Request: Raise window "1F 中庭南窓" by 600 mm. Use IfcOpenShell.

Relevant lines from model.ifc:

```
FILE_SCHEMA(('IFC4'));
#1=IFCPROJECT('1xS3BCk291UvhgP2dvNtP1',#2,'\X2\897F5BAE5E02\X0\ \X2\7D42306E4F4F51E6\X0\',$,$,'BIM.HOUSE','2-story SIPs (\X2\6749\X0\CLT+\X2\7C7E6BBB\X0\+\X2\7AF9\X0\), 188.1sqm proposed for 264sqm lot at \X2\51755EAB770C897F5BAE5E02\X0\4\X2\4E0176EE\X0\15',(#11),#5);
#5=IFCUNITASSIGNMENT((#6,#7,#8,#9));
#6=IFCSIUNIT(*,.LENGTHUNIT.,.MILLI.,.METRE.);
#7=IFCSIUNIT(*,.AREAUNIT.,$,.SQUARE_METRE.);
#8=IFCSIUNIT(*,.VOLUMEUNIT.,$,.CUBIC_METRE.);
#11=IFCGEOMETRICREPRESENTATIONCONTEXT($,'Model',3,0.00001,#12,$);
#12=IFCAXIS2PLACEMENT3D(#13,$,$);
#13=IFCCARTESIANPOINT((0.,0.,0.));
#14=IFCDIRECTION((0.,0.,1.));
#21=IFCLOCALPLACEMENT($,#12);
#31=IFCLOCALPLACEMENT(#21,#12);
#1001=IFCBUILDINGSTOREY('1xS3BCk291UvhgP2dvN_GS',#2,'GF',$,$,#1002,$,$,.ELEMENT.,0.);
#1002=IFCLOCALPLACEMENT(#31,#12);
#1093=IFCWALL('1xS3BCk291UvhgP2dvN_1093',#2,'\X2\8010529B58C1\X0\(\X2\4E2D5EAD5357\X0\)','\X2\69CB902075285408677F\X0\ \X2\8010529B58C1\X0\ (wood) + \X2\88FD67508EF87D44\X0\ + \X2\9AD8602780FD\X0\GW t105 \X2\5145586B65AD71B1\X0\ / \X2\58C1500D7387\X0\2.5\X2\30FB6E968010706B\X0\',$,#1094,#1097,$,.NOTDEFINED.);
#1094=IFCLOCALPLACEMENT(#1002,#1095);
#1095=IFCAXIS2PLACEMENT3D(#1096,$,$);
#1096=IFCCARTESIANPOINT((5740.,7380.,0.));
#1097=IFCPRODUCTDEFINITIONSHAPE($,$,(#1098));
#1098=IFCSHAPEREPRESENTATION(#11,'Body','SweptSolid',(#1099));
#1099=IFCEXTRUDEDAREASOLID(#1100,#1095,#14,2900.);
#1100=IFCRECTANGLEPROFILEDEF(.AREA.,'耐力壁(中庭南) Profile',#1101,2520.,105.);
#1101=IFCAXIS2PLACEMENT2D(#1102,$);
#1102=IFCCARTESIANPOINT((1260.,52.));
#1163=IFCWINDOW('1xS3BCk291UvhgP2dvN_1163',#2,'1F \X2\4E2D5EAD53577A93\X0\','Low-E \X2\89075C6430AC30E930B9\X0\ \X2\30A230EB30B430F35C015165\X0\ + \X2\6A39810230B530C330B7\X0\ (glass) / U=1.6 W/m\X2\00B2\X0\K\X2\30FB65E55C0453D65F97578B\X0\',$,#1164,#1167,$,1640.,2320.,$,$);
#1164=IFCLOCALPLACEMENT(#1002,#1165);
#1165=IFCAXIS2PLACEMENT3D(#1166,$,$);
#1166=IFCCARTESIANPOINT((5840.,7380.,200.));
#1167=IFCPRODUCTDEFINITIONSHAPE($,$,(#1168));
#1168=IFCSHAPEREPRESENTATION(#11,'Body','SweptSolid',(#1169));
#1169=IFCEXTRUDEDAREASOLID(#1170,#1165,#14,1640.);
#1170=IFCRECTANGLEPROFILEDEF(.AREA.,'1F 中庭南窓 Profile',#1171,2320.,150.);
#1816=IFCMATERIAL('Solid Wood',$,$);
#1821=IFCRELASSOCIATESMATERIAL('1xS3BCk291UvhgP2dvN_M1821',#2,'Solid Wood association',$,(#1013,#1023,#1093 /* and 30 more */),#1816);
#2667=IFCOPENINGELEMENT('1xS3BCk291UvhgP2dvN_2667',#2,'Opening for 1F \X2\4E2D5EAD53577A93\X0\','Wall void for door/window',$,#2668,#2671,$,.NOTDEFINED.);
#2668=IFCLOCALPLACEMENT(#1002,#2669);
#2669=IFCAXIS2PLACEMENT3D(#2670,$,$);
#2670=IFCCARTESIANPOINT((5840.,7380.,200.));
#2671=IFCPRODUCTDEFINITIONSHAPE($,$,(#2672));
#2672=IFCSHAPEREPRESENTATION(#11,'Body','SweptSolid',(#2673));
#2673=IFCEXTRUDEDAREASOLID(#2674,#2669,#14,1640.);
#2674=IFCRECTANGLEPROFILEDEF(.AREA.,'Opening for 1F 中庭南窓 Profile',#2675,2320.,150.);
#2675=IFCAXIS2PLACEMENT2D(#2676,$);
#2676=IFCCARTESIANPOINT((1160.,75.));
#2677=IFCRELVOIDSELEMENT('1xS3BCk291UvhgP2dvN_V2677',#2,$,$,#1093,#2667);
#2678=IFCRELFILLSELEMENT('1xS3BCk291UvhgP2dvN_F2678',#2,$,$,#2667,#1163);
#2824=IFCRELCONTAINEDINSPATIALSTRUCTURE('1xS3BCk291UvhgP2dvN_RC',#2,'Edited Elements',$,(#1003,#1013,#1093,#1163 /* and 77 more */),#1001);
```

```python
import numpy as np
import ifcopenshell
import ifcopenshell.api.geometry
import ifcopenshell.util.placement
import ifcopenshell.util.unit

model = ifcopenshell.open("model.ifc")
unit_scale = ifcopenshell.util.unit.calculate_unit_scale(model)

window = model.by_id(1163)
opening = window.FillsVoids[0].RelatingOpeningElement
dz = 0.6 / unit_scale

shift = np.array([0.0, 0.0, dz])
# The window is not placed relative to its opening, so move both.
for product in (opening, window):
    matrix = ifcopenshell.util.placement.get_local_placement(product.ObjectPlacement)
    matrix[:3, 3] += shift
    ifcopenshell.api.geometry.edit_object_placement(model, product=product, matrix=matrix, is_si=False)

print(f"moved by {dz * unit_scale:+.3f} m")

model.write("model-out.ifc")
```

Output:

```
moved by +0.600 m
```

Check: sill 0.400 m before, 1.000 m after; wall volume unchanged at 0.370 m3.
